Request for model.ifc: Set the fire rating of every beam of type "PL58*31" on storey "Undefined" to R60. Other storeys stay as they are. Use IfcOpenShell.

First a look at what the model holds.

```python
import ifcopenshell
import ifcopenshell.util.element

model = ifcopenshell.open("model.ifc")
print(model.schema)
storey = next(s for s in model.by_type("IfcBuildingStorey") if s.Name == "Undefined")
beams = [e for e in ifcopenshell.util.element.get_decomposition(storey) if e.is_a("IfcBeam")]
seen = {}
for e in beams:
    element_type = ifcopenshell.util.element.get_type(e)
    key = (element_type.Name if element_type != e and element_type else None, ifcopenshell.util.element.get_pset(e, "Pset_BeamCommon", "FireRating"))
    seen[key] = seen.get(key, 0) + 1
for (name, value), count in sorted(seen.items(), key=str):
    print(count, "x", name, "|", value)
```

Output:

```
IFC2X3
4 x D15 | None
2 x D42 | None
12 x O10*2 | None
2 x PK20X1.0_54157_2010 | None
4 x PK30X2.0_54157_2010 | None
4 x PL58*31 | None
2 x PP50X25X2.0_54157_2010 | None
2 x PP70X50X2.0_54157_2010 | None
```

```python
import ifcopenshell
import ifcopenshell.api.pset
import ifcopenshell.util.element

model = ifcopenshell.open("model.ifc")

storey = next(s for s in model.by_type("IfcBuildingStorey") if s.Name == "Undefined")
beams = [e for e in ifcopenshell.util.element.get_decomposition(storey) if e.is_a("IfcBeam")]

count = 0
for e in beams:
    element_type = ifcopenshell.util.element.get_type(e)
    if element_type in (None, e) or element_type.Name != "PL58*31":
        continue
    found = ifcopenshell.util.element.get_pset(e, "Pset_BeamCommon", should_inherit=False)
    if found:
        pset = model.by_id(found["id"])
        if len(ifcopenshell.util.element.get_elements_by_pset(pset)) > 1:
            pset = ifcopenshell.api.pset.unshare_pset(model, products=[e], pset=pset)[0]
    else:
        pset = ifcopenshell.api.pset.add_pset(model, product=e, name="Pset_BeamCommon")
    ifcopenshell.api.pset.edit_pset(model, pset=pset, properties={"FireRating": "R60"})
    count += 1

print(count, "beams updated")

model.write("model_v2.ifc")
```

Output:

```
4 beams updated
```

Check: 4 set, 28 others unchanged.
